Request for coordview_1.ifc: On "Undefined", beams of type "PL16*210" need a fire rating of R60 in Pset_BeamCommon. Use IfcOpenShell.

First a look at what the model holds.

```python
import ifcopenshell
import ifcopenshell.util.element

model = ifcopenshell.open("coordview_1.ifc")
print(model.schema)
storey = next(s for s in model.by_type("IfcBuildingStorey") if s.Name == "Undefined")
beams = [e for e in ifcopenshell.util.element.get_decomposition(storey) if e.is_a("IfcBeam")]
seen = {}
for e in beams:
    element_type = ifcopenshell.util.element.get_type(e)
    key = (element_type.Name if element_type != e and element_type else None, ifcopenshell.util.element.get_pset(e, "Pset_BeamCommon", "FireRating"))
    seen[key] = seen.get(key, 0) + 1
for (name, value), count in sorted(seen.items(), key=str):
    print(count, "x", name, "|", value)
```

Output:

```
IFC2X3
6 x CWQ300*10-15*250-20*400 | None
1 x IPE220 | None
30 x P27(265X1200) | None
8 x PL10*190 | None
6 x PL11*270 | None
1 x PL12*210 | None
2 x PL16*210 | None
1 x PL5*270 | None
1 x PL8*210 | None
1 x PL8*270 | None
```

```python
import ifcopenshell
import ifcopenshell.api.pset
import ifcopenshell.util.element

model = ifcopenshell.open("coordview_1.ifc")

storey = next(s for s in model.by_type("IfcBuildingStorey") if s.Name == "Undefined")
beams = [e for e in ifcopenshell.util.element.get_decomposition(storey) if e.is_a("IfcBeam")]

count = 0
for e in beams:
    element_type = ifcopenshell.util.element.get_type(e)
    if element_type in (None, e) or element_type.Name != "PL16*210":
        continue
    found = ifcopenshell.util.element.get_pset(e, "Pset_BeamCommon", should_inherit=False)
    if found:
        pset = model.by_id(found["id"])
        if len(ifcopenshell.util.element.get_elements_by_pset(pset)) > 1:
            pset = ifcopenshell.api.pset.unshare_pset(model, products=[e], pset=pset)[0]
    else:
        pset = ifcopenshell.api.pset.add_pset(model, product=e, name="Pset_BeamCommon")
    ifcopenshell.api.pset.edit_pset(model, pset=pset, properties={"FireRating": "R60"})
    count += 1

print(count, "beams updated")

model.write("coordview_1_updated.ifc")
```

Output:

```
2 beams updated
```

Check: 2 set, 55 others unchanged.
